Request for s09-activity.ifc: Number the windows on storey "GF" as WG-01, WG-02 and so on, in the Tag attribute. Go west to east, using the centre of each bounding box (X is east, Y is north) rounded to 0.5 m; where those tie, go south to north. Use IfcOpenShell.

First a look at what the model holds.

```python
import ifcopenshell
import ifcopenshell.util.element
import ifcopenshell.util.placement

model = ifcopenshell.open("s09-activity.ifc")
print(model.schema)
storey = next(s for s in model.by_type("IfcBuildingStorey") if s.Name == "GF")
windows = [e for e in ifcopenshell.util.element.get_decomposition(storey) if e.is_a("IfcWindow")]
for e in sorted(windows, key=lambda e: e.id()):
    origin = ifcopenshell.util.placement.get_local_placement(e.ObjectPlacement)[:3, 3]
    print(e.id(), e.Tag, e.Name, origin.round(2) + 0.0, sep=" | ")
```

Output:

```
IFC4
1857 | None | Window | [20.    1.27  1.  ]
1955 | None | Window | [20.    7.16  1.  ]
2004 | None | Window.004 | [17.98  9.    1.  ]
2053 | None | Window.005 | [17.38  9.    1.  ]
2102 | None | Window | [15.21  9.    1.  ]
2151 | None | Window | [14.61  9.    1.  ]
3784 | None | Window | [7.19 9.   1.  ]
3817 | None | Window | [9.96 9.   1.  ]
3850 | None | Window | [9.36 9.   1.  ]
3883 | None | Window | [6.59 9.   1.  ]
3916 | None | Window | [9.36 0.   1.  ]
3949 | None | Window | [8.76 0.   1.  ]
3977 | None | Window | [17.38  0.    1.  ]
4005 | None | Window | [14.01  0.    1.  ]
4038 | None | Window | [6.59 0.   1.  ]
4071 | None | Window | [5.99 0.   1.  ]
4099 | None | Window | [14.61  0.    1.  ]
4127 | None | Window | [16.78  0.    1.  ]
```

```python
import ifcopenshell
import ifcopenshell.geom
import ifcopenshell.util.element
import ifcopenshell.util.shape

model = ifcopenshell.open("s09-activity.ifc")
settings = ifcopenshell.geom.settings()
settings.set("use-world-coords", True)


def centre(element):
    shape = ifcopenshell.geom.create_shape(settings, element)
    return ifcopenshell.util.shape.get_bbox_centroid(shape.geometry)


storey = next(s for s in model.by_type("IfcBuildingStorey") if s.Name == "GF")
windows = [e for e in ifcopenshell.util.element.get_decomposition(storey) if e.is_a("IfcWindow")]

# Insertion points can sit at a corner or the storey origin, so sort by the geometry (in metres).
centres = {e: centre(e) for e in windows}
windows.sort(key=lambda e: (round(centres[e][0] / 0.5), centres[e][1]))

for i, e in enumerate(windows, start=1):
    number = f"WG-{i:02d}"
    e.Tag = number
    print(e.id(), number)

model.write("s09-activity-out.ifc")
```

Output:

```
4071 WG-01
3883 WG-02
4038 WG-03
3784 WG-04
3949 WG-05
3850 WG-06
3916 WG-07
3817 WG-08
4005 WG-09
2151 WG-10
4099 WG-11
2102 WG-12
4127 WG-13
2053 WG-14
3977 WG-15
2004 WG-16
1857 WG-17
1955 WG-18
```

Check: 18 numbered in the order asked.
